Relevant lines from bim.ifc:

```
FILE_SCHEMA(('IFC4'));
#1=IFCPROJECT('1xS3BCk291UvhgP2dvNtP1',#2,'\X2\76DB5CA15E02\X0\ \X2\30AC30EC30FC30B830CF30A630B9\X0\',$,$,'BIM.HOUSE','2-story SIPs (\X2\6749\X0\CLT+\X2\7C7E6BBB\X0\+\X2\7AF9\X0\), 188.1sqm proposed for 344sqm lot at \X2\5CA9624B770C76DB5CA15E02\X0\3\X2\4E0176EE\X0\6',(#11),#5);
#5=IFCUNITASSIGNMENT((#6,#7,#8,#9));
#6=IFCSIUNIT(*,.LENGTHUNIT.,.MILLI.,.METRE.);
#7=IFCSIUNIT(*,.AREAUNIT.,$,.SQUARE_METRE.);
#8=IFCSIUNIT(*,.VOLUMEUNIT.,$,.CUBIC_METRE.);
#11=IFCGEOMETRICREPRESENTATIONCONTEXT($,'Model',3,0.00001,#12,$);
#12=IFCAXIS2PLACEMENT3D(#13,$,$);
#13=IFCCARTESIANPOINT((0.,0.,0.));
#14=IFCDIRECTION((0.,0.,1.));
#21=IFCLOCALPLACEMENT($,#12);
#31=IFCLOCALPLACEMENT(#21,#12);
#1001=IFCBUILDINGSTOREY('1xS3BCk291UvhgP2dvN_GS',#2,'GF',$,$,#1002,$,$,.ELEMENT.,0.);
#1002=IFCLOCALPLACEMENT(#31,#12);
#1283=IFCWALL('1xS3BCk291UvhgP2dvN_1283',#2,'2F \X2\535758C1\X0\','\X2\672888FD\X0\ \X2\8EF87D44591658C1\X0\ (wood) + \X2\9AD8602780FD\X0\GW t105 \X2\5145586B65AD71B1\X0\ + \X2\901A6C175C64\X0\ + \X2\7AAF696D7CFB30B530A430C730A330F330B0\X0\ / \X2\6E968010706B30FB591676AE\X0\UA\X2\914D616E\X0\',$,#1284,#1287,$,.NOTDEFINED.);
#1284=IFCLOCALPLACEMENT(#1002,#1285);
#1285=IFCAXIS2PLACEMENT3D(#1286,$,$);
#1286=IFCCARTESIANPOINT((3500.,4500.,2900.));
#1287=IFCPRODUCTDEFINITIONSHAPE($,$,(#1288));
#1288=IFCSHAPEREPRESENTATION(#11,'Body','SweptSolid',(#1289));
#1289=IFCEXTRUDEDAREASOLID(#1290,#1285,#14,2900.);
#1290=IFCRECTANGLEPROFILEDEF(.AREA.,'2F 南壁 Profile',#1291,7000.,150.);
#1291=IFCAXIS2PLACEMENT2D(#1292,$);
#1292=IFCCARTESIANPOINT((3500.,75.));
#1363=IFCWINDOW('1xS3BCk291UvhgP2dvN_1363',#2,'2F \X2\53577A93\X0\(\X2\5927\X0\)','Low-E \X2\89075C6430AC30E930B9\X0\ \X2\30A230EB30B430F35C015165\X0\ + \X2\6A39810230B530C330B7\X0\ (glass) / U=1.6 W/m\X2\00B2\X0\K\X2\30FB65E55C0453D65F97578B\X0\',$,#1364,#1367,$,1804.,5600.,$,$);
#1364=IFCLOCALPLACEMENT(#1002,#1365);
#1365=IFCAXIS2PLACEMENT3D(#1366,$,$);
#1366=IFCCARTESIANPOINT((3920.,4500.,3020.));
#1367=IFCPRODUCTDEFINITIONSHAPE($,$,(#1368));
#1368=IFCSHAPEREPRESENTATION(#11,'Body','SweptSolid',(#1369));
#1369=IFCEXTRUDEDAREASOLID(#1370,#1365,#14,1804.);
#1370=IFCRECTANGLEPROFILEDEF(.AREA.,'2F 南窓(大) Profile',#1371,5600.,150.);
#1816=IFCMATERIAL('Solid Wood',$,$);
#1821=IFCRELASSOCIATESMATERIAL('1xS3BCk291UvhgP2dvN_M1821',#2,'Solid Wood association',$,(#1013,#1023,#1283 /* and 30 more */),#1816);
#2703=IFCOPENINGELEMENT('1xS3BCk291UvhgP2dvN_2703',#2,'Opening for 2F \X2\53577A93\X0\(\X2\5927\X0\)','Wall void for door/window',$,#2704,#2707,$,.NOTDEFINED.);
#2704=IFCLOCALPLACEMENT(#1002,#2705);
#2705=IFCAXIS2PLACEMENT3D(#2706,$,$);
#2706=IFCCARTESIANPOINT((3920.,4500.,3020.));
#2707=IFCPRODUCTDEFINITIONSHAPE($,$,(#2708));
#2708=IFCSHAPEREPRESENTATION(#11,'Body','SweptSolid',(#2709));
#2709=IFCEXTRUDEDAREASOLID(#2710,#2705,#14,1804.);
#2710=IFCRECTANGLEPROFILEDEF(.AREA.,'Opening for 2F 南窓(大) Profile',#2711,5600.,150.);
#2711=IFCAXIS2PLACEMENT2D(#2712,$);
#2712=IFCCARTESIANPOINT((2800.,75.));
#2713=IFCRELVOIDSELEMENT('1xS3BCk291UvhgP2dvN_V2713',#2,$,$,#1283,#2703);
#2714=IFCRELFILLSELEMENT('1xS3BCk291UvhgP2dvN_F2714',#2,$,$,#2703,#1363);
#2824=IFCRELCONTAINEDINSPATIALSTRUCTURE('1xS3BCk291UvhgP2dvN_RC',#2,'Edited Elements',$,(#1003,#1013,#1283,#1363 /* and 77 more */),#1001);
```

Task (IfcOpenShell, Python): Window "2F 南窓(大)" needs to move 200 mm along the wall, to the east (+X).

```python
import ifcopenshell
import ifcopenshell.api.geometry
import ifcopenshell.util.placement

model = ifcopenshell.open("bim.ifc")

window = model.by_guid("1xS3BCk291UvhgP2dvN_1363")
opening = window.FillsVoids[0].RelatingOpeningElement
wall = opening.VoidsElements[0].RelatingBuildingElement

wall_matrix = ifcopenshell.util.placement.get_local_placement(wall.ObjectPlacement)
shift = wall_matrix[:3, 0] * 200.0
before = ifcopenshell.util.placement.get_local_placement(window.ObjectPlacement)[:3, 3].copy()

# The window is not placed relative to its opening, so move both.
for product in (opening, window):
    matrix = ifcopenshell.util.placement.get_local_placement(product.ObjectPlacement)
    matrix[:3, 3] += shift
    ifcopenshell.api.geometry.edit_object_placement(model, product=product, matrix=matrix, is_si=False)

after = ifcopenshell.util.placement.get_local_placement(window.ObjectPlacement)[:3, 3]
print("window moved by", (after - before).round(3) + 0.0)

model.write("bim_rev.ifc")
```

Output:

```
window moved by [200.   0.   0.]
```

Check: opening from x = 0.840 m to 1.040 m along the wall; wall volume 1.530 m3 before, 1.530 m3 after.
